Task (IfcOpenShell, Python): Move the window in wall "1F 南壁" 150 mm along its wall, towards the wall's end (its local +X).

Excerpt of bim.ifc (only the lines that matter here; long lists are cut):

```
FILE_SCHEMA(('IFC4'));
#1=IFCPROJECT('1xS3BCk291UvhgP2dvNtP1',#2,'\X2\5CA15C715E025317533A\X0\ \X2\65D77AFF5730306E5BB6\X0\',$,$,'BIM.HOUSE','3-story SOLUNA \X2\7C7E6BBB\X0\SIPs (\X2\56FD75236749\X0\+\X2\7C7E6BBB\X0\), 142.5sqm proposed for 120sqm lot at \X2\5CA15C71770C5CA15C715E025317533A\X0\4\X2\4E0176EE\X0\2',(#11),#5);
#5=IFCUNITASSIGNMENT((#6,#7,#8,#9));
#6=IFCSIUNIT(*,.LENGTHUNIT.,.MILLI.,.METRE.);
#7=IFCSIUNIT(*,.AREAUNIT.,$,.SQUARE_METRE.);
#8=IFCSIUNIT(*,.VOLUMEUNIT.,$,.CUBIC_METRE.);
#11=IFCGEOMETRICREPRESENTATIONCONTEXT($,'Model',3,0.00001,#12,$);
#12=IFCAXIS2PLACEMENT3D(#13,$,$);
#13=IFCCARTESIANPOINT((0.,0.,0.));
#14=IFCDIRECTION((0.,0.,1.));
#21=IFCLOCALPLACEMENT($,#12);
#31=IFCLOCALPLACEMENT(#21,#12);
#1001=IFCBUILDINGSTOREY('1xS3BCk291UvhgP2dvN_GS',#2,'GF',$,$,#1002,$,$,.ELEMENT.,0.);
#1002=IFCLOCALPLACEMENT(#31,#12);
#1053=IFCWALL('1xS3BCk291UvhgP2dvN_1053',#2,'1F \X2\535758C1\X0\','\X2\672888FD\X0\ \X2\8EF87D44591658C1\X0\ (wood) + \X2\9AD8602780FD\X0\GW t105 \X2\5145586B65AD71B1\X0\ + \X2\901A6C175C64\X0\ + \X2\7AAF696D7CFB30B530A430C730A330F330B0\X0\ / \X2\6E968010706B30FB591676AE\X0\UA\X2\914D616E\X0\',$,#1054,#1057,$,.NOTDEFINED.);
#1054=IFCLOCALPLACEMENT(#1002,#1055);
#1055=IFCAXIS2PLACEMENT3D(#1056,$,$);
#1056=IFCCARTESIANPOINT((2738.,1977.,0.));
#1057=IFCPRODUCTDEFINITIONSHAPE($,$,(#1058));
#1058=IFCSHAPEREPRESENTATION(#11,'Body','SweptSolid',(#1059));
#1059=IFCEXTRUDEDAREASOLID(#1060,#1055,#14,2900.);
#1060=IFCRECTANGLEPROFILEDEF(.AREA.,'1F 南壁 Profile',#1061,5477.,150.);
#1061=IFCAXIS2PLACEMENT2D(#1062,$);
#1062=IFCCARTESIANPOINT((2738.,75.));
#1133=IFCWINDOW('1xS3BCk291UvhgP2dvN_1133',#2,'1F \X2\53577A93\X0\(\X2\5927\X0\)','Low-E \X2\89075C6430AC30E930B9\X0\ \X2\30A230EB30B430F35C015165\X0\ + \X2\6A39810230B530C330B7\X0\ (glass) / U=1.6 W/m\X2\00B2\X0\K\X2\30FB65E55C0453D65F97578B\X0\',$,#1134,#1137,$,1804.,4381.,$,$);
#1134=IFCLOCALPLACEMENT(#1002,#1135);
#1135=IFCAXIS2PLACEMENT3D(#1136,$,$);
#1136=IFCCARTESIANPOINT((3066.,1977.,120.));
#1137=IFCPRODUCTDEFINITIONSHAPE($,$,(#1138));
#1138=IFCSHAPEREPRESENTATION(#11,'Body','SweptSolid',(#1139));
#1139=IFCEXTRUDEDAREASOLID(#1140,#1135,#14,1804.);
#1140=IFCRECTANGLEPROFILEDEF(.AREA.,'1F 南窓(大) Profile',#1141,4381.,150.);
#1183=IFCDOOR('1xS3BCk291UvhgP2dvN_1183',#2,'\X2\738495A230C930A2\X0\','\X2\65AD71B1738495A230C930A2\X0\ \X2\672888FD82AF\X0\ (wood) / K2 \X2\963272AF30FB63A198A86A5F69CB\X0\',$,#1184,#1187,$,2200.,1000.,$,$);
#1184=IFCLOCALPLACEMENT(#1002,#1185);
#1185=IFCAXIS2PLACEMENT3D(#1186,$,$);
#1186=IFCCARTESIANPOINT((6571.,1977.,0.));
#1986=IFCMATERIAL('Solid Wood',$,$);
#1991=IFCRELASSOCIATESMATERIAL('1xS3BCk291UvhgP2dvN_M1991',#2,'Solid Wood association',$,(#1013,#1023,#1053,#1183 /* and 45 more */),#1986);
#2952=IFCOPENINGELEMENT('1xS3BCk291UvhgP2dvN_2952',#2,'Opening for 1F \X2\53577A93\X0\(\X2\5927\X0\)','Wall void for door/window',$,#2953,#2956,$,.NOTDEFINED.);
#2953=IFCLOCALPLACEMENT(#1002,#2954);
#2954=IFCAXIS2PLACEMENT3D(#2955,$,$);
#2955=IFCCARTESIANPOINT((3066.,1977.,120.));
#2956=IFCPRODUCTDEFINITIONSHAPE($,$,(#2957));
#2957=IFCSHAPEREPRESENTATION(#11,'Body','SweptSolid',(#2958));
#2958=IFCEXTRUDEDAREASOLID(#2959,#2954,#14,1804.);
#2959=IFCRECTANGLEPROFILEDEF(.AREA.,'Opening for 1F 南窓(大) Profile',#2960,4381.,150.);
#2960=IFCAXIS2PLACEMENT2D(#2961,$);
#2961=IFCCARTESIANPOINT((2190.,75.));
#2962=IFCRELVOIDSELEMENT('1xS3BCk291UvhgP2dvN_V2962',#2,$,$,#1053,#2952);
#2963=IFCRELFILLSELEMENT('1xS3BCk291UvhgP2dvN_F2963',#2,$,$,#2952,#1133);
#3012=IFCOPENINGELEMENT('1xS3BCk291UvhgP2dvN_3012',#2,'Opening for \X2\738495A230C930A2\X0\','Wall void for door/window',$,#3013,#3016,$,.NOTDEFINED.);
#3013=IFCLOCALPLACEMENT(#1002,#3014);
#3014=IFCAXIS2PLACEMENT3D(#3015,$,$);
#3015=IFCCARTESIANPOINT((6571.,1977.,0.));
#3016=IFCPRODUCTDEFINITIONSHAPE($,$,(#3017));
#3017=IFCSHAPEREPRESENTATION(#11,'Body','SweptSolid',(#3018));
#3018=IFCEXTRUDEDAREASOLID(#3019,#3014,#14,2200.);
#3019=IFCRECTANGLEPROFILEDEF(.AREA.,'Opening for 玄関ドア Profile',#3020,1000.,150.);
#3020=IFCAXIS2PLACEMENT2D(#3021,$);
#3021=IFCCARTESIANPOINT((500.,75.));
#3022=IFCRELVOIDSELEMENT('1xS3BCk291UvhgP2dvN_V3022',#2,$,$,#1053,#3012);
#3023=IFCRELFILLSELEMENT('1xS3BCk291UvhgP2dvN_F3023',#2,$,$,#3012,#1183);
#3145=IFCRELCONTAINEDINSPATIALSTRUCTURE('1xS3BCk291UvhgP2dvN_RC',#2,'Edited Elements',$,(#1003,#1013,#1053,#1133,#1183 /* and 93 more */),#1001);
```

```python
import ifcopenshell
import ifcopenshell.api.geometry
import ifcopenshell.util.placement
import ifcopenshell.util.unit

model = ifcopenshell.open("bim.ifc")
unit_scale = ifcopenshell.util.unit.calculate_unit_scale(model)

window = model.by_guid("1xS3BCk291UvhgP2dvN_1133")
opening = window.FillsVoids[0].RelatingOpeningElement
wall = opening.VoidsElements[0].RelatingBuildingElement

wall_matrix = ifcopenshell.util.placement.get_local_placement(wall.ObjectPlacement)
shift = wall_matrix[:3, 0] * 0.15 / unit_scale
before = ifcopenshell.util.placement.get_local_placement(window.ObjectPlacement)[:3, 3].copy()

# The window is not placed relative to its opening, so move both.
for product in (opening, window):
    matrix = ifcopenshell.util.placement.get_local_placement(product.ObjectPlacement)
    matrix[:3, 3] += shift
    ifcopenshell.api.geometry.edit_object_placement(model, product=product, matrix=matrix, is_si=False)

after = ifcopenshell.util.placement.get_local_placement(window.ObjectPlacement)[:3, 3]
print("window moved by", (after - before).round(3) + 0.0)

model.write("bim_updated.ifc")
```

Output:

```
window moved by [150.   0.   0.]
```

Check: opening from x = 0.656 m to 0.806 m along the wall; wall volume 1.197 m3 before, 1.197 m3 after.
